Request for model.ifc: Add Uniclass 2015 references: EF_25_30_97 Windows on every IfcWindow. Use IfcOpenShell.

First a look at what the model holds.

```python
import ifcopenshell

model = ifcopenshell.open("model.ifc")
print(model.schema)
print("classifications:", [c.Name for c in model.by_type("IfcClassification")])
for ifc_class in ("IfcDoor", "IfcRoof", "IfcStair", "IfcWall", "IfcWindow"):
    print(ifc_class, len(model.by_type(ifc_class)))
```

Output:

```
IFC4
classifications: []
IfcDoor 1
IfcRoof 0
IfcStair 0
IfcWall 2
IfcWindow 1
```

```python
import ifcopenshell
import ifcopenshell.api.classification

model = ifcopenshell.open("model.ifc")

system = ifcopenshell.api.classification.add_classification(model, classification="Uniclass 2015")

codes = {
    "IfcWindow": ("EF_25_30_97", "Windows"),
}
for ifc_class, (code, name) in codes.items():
    products = model.by_type(ifc_class)
    ifcopenshell.api.classification.add_reference(
        model, products=products, classification=system, identification=code, name=name
    )
    print(code, len(products))

model.write("model-out.ifc")
```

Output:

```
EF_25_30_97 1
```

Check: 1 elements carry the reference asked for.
